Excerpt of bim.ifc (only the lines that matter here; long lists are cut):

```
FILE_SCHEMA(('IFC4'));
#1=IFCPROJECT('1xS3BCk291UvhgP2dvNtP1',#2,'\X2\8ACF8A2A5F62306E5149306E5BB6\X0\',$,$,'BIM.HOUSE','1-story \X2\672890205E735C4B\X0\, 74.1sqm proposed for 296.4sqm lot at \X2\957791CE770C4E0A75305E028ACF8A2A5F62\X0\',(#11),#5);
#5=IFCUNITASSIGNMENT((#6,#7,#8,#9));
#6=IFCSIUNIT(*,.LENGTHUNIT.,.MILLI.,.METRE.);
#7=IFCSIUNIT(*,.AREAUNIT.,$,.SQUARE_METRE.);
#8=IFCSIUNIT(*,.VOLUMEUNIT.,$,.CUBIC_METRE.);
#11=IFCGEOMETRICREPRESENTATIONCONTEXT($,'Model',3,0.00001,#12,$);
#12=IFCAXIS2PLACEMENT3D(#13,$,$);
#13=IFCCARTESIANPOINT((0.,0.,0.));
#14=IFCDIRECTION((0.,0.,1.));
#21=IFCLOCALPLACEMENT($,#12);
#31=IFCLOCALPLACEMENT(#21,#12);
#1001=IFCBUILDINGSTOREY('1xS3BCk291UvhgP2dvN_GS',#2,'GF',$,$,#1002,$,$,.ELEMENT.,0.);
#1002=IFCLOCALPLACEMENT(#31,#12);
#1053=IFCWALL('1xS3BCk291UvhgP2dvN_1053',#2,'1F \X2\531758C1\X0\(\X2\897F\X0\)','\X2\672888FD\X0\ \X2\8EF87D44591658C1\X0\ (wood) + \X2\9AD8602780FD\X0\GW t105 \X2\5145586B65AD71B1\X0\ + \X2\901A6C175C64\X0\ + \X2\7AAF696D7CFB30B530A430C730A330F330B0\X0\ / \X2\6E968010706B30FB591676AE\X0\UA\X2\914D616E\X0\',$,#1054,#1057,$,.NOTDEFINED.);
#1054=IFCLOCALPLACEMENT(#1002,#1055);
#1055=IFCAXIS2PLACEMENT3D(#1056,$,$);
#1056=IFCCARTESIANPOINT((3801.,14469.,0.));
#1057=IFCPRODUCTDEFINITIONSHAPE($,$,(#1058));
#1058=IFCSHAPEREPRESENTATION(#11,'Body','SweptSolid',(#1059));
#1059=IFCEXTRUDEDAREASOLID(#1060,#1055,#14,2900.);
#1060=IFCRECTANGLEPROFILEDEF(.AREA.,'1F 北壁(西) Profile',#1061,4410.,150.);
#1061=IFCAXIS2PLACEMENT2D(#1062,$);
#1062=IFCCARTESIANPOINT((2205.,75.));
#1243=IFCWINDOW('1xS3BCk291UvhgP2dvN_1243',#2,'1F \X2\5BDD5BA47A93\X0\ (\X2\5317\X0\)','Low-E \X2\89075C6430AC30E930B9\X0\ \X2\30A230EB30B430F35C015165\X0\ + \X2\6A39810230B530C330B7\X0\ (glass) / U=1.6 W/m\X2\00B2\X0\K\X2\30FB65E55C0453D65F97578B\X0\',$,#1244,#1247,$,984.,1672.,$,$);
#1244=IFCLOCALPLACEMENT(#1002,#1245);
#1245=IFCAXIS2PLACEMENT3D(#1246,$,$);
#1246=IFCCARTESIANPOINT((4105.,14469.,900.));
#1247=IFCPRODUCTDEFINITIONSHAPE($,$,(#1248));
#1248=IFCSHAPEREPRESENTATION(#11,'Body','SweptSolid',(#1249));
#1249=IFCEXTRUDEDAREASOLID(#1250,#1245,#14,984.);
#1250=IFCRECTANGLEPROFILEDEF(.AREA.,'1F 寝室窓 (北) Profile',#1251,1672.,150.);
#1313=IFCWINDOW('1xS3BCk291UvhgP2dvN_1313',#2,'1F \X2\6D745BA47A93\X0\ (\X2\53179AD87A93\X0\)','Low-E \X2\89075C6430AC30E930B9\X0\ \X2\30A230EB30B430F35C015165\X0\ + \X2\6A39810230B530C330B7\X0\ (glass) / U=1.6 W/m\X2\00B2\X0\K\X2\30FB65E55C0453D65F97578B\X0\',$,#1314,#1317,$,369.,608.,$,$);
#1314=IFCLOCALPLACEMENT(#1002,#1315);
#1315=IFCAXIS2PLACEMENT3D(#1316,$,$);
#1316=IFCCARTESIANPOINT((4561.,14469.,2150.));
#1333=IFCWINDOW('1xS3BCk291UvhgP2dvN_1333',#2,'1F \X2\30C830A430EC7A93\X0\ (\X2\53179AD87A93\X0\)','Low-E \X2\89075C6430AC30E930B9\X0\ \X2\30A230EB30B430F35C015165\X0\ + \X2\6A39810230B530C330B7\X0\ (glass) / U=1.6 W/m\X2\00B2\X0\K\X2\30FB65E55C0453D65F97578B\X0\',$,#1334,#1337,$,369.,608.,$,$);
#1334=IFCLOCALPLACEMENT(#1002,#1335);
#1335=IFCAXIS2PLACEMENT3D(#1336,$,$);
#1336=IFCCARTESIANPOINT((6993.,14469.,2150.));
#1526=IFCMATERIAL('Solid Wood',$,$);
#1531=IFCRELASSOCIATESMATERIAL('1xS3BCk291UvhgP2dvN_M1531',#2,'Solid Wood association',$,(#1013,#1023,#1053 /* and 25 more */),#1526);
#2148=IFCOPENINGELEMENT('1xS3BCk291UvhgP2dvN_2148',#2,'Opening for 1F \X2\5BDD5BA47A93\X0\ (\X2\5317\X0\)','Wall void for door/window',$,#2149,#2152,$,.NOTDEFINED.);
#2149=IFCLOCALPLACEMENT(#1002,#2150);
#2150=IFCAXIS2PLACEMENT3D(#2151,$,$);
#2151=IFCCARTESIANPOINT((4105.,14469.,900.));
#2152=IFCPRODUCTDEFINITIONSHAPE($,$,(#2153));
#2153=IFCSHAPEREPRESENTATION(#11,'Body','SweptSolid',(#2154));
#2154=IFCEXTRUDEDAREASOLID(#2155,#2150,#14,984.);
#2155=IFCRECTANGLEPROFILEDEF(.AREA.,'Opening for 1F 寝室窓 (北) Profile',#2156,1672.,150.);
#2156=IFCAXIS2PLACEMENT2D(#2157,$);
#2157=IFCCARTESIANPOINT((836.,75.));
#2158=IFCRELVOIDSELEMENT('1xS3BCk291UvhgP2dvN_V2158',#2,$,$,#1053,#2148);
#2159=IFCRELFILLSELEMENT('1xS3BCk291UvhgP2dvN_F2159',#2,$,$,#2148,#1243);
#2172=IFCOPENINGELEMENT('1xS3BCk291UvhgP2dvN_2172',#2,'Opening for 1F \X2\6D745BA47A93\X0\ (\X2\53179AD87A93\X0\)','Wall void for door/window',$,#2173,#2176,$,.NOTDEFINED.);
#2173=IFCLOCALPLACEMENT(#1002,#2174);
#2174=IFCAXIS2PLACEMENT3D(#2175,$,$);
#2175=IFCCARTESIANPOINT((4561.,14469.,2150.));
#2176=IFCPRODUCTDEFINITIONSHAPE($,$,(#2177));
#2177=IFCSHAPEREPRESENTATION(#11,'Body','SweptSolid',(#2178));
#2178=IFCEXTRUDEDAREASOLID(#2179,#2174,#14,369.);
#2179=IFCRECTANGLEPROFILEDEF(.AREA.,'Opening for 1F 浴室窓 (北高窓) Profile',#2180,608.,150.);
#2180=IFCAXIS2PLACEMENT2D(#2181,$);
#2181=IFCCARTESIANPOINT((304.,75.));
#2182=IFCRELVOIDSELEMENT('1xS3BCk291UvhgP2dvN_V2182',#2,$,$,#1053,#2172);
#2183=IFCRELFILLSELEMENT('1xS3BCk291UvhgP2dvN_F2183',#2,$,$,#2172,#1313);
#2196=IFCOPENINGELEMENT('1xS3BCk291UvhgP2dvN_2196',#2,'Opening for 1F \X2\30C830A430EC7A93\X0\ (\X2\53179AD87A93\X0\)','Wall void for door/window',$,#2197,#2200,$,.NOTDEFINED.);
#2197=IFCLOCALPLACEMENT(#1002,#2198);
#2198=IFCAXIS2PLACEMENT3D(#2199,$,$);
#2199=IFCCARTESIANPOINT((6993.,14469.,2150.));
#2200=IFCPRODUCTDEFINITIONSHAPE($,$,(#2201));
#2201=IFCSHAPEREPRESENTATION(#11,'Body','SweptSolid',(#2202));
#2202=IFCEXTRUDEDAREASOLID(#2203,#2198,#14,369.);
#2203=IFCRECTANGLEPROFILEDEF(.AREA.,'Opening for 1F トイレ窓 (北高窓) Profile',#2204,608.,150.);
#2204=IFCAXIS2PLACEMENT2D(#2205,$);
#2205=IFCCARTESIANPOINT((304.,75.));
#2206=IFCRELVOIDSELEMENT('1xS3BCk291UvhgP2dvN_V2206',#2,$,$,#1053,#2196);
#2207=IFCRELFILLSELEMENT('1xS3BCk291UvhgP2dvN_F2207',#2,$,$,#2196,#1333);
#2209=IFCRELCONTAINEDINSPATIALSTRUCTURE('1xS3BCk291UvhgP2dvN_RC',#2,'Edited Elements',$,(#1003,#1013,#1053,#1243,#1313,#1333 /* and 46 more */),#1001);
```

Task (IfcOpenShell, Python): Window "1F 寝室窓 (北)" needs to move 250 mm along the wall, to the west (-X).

```python
import ifcopenshell
import ifcopenshell.api.geometry
import ifcopenshell.util.placement
import ifcopenshell.util.unit

model = ifcopenshell.open("bim.ifc")
unit_scale = ifcopenshell.util.unit.calculate_unit_scale(model)

window = model.by_guid("1xS3BCk291UvhgP2dvN_1243")
opening = window.FillsVoids[0].RelatingOpeningElement
wall = opening.VoidsElements[0].RelatingBuildingElement

wall_matrix = ifcopenshell.util.placement.get_local_placement(wall.ObjectPlacement)
shift = wall_matrix[:3, 0] * -0.25 / unit_scale
before = ifcopenshell.util.placement.get_local_placement(window.ObjectPlacement)[:3, 3].copy()

# The window is not placed relative to its opening, so move both.
for product in (opening, window):
    matrix = ifcopenshell.util.placement.get_local_placement(product.ObjectPlacement)
    matrix[:3, 3] += shift
    ifcopenshell.api.geometry.edit_object_placement(model, product=product, matrix=matrix, is_si=False)

after = ifcopenshell.util.placement.get_local_placement(window.ObjectPlacement)[:3, 3]
print("window moved by", (after - before).round(3) + 0.0)

model.write("bim_rev.ifc")
```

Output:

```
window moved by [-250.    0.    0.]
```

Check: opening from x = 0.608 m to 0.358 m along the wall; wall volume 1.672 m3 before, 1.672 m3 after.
